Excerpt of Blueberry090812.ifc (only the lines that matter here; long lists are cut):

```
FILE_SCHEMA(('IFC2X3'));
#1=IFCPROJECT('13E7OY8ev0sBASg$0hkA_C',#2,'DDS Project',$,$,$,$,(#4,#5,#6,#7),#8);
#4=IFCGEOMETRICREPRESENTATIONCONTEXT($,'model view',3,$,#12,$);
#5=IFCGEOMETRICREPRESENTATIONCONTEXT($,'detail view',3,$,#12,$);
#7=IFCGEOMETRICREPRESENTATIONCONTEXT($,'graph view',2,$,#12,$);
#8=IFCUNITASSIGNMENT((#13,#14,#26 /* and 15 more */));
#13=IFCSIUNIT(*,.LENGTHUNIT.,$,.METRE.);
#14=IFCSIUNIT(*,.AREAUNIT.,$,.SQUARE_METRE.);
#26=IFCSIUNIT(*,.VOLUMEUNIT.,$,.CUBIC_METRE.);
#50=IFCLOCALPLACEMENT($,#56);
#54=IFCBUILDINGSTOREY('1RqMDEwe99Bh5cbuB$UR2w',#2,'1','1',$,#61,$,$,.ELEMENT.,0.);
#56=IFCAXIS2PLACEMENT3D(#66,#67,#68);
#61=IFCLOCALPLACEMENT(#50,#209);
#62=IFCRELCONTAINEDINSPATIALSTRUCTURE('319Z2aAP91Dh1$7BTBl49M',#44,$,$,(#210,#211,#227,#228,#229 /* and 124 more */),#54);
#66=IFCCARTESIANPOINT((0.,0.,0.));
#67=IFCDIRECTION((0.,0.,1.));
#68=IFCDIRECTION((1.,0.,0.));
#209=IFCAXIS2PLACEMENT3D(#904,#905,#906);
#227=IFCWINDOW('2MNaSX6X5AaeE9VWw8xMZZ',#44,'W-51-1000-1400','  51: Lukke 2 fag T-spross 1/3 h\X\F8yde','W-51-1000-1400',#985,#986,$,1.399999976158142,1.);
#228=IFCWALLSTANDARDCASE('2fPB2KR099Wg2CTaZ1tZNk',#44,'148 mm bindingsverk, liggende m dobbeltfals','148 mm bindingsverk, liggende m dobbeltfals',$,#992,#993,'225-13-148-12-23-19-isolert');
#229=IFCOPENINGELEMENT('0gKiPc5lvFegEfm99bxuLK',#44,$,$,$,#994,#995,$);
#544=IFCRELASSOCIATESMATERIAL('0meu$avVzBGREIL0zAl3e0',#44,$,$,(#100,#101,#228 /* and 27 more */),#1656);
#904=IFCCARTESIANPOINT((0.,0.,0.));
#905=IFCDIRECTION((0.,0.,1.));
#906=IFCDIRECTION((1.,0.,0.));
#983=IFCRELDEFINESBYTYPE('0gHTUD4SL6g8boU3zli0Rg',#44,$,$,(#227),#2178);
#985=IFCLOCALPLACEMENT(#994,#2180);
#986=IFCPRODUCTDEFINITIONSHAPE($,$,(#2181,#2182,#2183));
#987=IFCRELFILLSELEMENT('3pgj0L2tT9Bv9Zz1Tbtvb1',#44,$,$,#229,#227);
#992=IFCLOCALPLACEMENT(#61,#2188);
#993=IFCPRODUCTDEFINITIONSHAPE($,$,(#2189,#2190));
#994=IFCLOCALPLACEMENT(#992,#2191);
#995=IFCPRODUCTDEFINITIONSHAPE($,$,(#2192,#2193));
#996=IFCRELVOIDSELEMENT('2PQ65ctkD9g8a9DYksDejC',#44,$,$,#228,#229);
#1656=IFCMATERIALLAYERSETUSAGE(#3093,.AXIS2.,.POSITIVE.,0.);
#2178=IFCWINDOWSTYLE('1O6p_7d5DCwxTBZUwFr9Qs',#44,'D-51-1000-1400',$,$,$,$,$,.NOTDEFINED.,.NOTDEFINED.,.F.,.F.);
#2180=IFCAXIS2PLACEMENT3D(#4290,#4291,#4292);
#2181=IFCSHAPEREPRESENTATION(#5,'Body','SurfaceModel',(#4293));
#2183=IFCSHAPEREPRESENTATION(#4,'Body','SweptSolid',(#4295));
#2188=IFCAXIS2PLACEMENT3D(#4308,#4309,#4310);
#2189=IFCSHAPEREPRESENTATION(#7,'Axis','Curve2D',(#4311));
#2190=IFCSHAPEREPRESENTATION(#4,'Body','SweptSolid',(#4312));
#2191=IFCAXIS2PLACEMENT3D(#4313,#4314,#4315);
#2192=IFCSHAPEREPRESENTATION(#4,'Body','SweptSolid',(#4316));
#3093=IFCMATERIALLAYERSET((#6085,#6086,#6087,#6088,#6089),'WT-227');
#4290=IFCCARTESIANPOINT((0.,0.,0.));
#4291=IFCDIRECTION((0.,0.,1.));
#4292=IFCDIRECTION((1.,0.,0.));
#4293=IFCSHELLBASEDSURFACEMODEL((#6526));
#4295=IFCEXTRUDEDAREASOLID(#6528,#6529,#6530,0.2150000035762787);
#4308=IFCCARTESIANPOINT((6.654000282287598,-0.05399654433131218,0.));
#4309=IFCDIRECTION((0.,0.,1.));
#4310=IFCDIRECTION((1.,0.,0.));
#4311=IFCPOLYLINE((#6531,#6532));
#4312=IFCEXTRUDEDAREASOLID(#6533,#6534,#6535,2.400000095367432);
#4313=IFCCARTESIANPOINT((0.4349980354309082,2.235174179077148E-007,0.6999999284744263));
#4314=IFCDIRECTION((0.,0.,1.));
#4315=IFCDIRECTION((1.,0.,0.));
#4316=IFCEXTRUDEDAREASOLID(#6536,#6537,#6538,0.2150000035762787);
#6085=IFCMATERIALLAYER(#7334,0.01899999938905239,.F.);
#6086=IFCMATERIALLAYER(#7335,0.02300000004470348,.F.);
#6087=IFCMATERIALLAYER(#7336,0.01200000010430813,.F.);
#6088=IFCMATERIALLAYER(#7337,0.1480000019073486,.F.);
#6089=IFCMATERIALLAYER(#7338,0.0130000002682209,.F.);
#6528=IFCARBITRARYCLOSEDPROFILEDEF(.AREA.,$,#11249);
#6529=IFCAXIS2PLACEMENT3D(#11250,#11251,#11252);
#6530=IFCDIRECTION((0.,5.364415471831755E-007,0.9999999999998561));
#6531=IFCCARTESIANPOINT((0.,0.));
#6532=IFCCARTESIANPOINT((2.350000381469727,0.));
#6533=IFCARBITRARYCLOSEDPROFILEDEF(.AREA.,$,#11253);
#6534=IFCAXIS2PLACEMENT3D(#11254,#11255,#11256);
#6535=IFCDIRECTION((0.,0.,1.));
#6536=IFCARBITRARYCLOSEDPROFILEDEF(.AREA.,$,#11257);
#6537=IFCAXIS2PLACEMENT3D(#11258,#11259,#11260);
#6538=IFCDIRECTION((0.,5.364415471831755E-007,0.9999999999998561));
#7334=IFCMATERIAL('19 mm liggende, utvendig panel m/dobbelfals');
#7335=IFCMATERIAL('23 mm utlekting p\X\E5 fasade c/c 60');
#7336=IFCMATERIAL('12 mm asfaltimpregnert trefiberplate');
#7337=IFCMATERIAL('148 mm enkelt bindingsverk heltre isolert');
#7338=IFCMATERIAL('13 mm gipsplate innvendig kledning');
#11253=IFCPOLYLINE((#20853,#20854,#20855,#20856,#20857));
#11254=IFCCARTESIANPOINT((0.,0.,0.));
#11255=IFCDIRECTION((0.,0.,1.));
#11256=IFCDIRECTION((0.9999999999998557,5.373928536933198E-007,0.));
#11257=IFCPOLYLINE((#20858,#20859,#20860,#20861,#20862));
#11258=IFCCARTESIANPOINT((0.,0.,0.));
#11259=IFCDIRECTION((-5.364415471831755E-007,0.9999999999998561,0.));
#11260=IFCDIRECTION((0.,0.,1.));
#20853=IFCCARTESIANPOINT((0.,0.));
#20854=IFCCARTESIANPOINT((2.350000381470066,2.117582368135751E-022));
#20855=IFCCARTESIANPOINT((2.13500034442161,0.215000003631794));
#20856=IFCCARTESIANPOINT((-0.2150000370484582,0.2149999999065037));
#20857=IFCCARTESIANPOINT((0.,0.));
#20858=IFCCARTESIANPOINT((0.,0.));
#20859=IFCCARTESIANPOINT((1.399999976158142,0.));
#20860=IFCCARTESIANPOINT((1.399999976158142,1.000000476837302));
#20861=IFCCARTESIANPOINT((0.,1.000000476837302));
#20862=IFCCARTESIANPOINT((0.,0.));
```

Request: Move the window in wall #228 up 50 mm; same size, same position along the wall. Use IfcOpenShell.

```python
import numpy as np
import ifcopenshell
import ifcopenshell.api.geometry
import ifcopenshell.util.placement
import ifcopenshell.util.unit

model = ifcopenshell.open("Blueberry090812.ifc")
unit_scale = ifcopenshell.util.unit.calculate_unit_scale(model)

window = model.by_guid("2MNaSX6X5AaeE9VWw8xMZZ")
opening = window.FillsVoids[0].RelatingOpeningElement
dz = 0.05

shift = np.array([0.0, 0.0, dz])
# The window is placed relative to its opening, so it follows when the opening moves.
matrix = ifcopenshell.util.placement.get_local_placement(opening.ObjectPlacement)
matrix[:3, 3] += shift
ifcopenshell.api.geometry.edit_object_placement(
    model, product=opening, matrix=matrix, is_si=False, should_transform_children=True
)

print(f"moved by {dz * unit_scale:+.3f} m")

model.write("Blueberry090812_edited.ifc")
```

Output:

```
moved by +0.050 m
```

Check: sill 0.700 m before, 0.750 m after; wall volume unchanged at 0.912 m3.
